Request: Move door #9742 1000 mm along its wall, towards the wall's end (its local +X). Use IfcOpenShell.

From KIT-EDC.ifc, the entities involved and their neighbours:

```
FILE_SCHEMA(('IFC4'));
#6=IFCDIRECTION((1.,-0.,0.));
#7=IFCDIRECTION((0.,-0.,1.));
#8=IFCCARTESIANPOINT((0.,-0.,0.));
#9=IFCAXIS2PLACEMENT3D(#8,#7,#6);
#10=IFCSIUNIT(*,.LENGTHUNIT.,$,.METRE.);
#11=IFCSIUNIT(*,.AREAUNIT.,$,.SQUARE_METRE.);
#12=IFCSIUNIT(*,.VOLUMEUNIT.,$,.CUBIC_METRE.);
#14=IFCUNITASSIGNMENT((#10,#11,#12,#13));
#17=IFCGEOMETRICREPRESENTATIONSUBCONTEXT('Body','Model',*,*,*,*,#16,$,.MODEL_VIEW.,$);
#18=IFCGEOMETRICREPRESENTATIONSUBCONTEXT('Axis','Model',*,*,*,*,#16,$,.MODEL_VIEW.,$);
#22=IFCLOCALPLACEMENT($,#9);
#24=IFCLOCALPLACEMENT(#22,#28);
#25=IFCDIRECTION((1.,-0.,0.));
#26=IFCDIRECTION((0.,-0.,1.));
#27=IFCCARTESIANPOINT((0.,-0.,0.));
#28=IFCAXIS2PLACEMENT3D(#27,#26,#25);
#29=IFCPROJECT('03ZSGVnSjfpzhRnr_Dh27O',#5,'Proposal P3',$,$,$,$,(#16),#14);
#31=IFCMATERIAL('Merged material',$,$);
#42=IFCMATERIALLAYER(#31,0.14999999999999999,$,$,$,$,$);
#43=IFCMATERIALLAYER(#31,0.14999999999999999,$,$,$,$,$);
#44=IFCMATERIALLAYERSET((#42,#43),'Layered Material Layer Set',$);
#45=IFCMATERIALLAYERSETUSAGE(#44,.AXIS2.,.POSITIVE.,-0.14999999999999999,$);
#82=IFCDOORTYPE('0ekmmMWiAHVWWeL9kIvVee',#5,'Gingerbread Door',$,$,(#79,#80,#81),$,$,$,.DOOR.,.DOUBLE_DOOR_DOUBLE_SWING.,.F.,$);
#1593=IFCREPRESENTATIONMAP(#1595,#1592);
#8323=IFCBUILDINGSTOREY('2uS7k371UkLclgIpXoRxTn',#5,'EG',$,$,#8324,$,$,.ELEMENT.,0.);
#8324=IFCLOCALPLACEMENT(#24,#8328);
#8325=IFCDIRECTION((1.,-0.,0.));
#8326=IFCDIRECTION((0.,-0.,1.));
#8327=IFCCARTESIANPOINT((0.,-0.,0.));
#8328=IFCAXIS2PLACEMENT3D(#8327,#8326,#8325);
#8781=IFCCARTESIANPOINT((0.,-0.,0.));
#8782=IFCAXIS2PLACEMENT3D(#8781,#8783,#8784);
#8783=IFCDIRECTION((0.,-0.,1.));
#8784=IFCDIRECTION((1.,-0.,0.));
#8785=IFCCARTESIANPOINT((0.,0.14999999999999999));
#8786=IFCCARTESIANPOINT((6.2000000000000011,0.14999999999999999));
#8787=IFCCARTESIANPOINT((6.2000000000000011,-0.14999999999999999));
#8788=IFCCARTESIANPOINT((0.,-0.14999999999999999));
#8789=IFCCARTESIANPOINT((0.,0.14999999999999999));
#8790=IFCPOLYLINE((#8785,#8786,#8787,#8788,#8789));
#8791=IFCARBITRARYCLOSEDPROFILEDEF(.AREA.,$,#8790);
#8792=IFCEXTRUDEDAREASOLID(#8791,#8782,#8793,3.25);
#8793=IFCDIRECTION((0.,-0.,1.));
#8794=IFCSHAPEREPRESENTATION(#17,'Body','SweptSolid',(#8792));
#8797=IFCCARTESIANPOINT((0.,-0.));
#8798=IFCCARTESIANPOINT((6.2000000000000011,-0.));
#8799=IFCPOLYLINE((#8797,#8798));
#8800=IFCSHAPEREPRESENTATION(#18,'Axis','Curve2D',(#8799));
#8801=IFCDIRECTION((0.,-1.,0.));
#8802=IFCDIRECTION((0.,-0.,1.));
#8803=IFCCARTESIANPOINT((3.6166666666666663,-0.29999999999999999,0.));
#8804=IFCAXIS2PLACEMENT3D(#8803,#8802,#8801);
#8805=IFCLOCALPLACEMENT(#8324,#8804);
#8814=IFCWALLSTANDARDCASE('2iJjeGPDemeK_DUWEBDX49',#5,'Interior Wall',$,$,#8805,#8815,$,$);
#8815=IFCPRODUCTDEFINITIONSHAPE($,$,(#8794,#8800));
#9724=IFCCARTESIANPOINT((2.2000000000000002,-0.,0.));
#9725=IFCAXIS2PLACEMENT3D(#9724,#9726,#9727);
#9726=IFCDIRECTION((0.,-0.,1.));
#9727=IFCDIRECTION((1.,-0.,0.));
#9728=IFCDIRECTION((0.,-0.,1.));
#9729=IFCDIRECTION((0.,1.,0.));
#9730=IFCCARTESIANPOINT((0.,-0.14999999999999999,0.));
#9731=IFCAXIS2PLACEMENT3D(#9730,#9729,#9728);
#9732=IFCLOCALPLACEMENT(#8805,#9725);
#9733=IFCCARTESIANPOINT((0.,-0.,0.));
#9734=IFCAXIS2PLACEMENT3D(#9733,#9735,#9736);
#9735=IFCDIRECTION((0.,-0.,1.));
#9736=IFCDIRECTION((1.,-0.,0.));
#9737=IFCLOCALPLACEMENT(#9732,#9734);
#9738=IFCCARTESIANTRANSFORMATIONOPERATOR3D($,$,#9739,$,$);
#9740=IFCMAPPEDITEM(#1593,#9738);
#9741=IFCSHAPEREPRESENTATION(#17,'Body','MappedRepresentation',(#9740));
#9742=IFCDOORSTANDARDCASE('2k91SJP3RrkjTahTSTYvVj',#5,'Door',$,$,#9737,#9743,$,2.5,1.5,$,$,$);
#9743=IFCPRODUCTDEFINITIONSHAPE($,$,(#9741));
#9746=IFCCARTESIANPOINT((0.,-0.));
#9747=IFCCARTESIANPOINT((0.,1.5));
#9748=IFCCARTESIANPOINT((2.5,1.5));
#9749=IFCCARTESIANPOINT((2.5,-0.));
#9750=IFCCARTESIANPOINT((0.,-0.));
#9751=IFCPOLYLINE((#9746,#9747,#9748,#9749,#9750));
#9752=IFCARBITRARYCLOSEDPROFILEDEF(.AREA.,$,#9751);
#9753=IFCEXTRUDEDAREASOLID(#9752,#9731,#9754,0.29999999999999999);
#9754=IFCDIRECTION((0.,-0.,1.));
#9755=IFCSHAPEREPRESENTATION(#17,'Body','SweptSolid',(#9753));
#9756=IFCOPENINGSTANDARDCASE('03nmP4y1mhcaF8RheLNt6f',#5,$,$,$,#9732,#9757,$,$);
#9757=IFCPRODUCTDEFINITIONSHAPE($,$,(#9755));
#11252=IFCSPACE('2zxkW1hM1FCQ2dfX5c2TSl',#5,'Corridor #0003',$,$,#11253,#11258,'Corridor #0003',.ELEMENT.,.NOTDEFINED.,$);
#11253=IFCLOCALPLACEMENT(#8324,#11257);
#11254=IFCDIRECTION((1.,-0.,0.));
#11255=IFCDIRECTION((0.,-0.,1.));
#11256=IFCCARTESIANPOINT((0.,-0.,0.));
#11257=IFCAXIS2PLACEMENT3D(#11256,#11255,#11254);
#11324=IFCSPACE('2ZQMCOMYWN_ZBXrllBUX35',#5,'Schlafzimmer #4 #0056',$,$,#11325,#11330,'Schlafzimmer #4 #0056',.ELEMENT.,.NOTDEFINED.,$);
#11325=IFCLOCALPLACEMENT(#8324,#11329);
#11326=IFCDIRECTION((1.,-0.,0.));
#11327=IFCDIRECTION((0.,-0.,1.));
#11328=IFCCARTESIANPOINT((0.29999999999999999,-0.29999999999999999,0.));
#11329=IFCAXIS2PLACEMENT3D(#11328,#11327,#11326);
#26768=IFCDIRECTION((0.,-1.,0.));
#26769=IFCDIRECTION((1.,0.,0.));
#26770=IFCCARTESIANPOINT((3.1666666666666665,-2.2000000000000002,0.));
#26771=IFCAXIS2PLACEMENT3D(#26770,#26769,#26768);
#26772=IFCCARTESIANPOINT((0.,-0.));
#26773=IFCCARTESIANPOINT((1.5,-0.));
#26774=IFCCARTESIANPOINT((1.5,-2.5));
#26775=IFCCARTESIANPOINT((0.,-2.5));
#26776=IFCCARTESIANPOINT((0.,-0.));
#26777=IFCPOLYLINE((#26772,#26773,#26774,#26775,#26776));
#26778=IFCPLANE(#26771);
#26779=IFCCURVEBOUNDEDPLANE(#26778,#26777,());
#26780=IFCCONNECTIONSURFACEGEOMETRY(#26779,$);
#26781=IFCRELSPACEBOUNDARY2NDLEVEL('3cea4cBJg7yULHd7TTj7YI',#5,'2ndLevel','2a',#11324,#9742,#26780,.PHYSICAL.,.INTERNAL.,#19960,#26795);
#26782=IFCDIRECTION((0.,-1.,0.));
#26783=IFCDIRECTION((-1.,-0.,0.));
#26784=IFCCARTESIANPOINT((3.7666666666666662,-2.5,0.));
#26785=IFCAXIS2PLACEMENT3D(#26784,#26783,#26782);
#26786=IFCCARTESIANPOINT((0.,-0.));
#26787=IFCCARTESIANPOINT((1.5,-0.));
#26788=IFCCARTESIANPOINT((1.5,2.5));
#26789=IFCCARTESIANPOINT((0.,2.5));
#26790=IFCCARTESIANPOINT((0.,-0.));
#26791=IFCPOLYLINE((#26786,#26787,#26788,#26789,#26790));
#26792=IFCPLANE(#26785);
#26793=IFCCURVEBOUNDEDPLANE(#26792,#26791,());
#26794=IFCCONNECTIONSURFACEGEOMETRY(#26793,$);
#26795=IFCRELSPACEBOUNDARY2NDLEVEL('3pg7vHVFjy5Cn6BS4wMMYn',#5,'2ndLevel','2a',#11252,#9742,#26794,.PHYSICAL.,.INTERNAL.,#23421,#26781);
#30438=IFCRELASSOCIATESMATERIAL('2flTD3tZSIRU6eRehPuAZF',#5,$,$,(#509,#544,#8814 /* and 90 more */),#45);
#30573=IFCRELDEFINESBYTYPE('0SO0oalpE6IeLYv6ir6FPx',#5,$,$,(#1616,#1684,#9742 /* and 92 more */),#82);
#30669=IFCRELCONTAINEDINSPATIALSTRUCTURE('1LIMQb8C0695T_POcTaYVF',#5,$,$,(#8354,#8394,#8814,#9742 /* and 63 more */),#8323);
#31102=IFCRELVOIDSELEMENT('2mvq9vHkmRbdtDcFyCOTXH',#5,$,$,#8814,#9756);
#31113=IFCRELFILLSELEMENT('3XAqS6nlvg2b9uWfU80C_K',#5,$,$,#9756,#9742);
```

```python
import numpy as np
import ifcopenshell
import ifcopenshell.api.geometry
import ifcopenshell.util.placement

model = ifcopenshell.open("KIT-EDC.ifc")

door = model.by_id(9742)
opening = door.FillsVoids[0].RelatingOpeningElement
wall = opening.VoidsElements[0].RelatingBuildingElement

wall_matrix = ifcopenshell.util.placement.get_local_placement(wall.ObjectPlacement)
shift = wall_matrix[:3, 0] * 1.0
before = ifcopenshell.util.placement.get_local_placement(door.ObjectPlacement)[:3, 3].copy()

# The door is placed relative to its opening, so it follows when the opening moves.
matrix = ifcopenshell.util.placement.get_local_placement(opening.ObjectPlacement)
matrix[:3, 3] += shift
ifcopenshell.api.geometry.edit_object_placement(
    model, product=opening, matrix=matrix, is_si=False, should_transform_children=True
)

# Space boundary surfaces are stored in each space's coordinates; move them too.
for rel in door.ProvidesBoundaries:
    if not rel.ConnectionGeometry:
        continue
    surface = rel.ConnectionGeometry.SurfaceOnRelatingElement.BasisSurface
    space_matrix = ifcopenshell.util.placement.get_local_placement(rel.RelatingSpace.ObjectPlacement)
    point = np.array(surface.Position.Location.Coordinates) + space_matrix[:3, :3].T @ shift
    surface.Position = model.createIfcAxis2Placement3D(
        model.createIfcCartesianPoint(point.tolist()), surface.Position.Axis, surface.Position.RefDirection
    )

after = ifcopenshell.util.placement.get_local_placement(door.ObjectPlacement)[:3, 3]
print("door moved by", (after - before).round(3) + 0.0)

model.write("KIT-EDC_updated.ifc")
```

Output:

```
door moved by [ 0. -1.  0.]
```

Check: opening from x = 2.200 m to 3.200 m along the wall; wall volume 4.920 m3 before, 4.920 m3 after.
